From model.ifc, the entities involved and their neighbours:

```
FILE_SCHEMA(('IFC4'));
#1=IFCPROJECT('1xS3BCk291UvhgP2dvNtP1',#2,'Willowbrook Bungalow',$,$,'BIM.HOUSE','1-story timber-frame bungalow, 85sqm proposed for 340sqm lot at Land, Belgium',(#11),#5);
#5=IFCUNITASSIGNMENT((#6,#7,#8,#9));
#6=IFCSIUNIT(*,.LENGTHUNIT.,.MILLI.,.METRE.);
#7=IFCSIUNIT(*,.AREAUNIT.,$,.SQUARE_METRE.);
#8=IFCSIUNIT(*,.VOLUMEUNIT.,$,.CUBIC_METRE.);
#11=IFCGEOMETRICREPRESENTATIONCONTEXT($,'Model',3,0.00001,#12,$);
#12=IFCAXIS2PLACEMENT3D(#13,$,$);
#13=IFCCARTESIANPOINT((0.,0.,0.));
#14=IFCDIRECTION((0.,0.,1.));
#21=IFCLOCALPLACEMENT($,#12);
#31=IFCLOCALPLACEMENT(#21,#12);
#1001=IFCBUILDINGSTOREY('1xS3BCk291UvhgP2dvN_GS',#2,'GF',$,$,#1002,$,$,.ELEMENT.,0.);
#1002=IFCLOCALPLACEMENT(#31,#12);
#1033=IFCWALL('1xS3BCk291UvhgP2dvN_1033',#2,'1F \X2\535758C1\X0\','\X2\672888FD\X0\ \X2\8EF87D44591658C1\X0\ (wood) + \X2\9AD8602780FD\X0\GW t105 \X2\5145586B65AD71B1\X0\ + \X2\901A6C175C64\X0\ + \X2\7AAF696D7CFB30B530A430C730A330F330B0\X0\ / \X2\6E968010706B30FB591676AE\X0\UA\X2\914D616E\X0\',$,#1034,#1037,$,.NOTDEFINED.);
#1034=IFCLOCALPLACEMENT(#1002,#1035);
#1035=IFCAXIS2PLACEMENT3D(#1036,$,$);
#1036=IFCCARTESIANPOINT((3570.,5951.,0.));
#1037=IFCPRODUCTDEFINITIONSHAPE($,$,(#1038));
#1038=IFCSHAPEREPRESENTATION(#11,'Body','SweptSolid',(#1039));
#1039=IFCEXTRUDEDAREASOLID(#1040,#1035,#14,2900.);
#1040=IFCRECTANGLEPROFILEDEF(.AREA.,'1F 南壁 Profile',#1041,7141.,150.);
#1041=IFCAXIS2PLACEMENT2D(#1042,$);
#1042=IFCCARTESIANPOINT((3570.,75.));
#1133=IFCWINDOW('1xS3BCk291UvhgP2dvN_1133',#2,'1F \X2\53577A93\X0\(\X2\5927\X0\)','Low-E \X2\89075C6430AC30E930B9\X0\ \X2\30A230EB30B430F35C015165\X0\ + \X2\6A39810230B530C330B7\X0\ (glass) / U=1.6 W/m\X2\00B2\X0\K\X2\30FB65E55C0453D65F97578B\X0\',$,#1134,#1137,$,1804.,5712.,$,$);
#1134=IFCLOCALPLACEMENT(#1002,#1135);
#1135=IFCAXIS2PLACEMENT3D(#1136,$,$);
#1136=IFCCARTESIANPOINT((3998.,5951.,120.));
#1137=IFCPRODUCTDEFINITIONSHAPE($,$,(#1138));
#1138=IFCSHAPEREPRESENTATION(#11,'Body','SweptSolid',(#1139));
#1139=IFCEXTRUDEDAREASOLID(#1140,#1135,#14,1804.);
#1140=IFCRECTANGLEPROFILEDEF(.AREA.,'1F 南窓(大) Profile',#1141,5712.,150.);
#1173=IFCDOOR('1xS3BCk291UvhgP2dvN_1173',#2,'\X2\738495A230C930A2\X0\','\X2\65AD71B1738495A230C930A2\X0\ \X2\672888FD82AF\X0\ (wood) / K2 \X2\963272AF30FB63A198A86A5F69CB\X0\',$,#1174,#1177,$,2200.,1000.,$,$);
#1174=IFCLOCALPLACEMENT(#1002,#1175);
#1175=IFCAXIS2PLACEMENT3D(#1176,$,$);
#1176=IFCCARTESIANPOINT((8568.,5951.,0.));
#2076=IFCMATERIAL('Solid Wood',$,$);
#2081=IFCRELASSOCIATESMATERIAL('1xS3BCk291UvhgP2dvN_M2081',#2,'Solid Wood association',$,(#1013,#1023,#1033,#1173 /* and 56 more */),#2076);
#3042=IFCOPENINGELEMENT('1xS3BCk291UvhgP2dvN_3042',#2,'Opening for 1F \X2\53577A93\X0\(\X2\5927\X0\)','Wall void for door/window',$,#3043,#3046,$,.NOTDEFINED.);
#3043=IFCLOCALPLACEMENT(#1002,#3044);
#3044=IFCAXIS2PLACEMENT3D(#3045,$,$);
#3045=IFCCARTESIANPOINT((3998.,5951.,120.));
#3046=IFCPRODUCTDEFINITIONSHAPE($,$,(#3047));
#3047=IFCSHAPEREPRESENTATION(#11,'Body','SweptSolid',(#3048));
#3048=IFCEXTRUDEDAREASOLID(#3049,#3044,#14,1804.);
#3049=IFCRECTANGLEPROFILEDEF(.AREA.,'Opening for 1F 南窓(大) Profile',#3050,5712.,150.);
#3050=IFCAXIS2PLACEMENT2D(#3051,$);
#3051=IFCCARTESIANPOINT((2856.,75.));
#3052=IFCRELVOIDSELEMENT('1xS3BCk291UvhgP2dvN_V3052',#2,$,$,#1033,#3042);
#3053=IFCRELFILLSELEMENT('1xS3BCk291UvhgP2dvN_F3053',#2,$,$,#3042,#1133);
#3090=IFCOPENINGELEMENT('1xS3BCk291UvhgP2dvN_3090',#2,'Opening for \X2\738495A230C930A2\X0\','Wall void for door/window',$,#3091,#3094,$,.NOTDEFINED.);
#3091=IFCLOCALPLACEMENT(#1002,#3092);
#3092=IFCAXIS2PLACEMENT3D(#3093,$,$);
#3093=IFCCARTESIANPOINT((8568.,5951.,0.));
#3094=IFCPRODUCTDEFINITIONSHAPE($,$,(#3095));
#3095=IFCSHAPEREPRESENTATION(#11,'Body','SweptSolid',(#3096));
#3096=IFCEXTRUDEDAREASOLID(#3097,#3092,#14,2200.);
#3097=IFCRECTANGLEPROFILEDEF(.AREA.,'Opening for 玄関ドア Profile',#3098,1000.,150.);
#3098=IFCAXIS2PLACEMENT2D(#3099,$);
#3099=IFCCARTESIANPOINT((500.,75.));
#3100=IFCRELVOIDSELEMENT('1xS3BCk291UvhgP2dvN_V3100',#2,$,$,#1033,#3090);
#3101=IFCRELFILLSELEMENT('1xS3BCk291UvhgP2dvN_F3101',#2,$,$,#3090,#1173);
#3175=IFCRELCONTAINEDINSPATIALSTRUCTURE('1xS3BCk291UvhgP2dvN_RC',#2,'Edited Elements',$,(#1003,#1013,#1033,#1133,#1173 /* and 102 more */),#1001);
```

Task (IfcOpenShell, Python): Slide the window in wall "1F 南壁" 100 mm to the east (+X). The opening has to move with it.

```python
import ifcopenshell
import ifcopenshell.api.geometry
import ifcopenshell.util.placement

model = ifcopenshell.open("model.ifc")

window = model.by_guid("1xS3BCk291UvhgP2dvN_1133")
opening = window.FillsVoids[0].RelatingOpeningElement
wall = opening.VoidsElements[0].RelatingBuildingElement

wall_matrix = ifcopenshell.util.placement.get_local_placement(wall.ObjectPlacement)
shift = wall_matrix[:3, 0] * 100.0
before = ifcopenshell.util.placement.get_local_placement(window.ObjectPlacement)[:3, 3].copy()

# The window is not placed relative to its opening, so move both.
for product in (opening, window):
    matrix = ifcopenshell.util.placement.get_local_placement(product.ObjectPlacement)
    matrix[:3, 3] += shift
    ifcopenshell.api.geometry.edit_object_placement(model, product=product, matrix=matrix, is_si=False)

after = ifcopenshell.util.placement.get_local_placement(window.ObjectPlacement)[:3, 3]
print("window moved by", (after - before).round(3) + 0.0)

model.write("model_updated.ifc")
```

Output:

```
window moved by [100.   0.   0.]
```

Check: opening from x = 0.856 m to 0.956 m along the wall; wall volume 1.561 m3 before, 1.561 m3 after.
